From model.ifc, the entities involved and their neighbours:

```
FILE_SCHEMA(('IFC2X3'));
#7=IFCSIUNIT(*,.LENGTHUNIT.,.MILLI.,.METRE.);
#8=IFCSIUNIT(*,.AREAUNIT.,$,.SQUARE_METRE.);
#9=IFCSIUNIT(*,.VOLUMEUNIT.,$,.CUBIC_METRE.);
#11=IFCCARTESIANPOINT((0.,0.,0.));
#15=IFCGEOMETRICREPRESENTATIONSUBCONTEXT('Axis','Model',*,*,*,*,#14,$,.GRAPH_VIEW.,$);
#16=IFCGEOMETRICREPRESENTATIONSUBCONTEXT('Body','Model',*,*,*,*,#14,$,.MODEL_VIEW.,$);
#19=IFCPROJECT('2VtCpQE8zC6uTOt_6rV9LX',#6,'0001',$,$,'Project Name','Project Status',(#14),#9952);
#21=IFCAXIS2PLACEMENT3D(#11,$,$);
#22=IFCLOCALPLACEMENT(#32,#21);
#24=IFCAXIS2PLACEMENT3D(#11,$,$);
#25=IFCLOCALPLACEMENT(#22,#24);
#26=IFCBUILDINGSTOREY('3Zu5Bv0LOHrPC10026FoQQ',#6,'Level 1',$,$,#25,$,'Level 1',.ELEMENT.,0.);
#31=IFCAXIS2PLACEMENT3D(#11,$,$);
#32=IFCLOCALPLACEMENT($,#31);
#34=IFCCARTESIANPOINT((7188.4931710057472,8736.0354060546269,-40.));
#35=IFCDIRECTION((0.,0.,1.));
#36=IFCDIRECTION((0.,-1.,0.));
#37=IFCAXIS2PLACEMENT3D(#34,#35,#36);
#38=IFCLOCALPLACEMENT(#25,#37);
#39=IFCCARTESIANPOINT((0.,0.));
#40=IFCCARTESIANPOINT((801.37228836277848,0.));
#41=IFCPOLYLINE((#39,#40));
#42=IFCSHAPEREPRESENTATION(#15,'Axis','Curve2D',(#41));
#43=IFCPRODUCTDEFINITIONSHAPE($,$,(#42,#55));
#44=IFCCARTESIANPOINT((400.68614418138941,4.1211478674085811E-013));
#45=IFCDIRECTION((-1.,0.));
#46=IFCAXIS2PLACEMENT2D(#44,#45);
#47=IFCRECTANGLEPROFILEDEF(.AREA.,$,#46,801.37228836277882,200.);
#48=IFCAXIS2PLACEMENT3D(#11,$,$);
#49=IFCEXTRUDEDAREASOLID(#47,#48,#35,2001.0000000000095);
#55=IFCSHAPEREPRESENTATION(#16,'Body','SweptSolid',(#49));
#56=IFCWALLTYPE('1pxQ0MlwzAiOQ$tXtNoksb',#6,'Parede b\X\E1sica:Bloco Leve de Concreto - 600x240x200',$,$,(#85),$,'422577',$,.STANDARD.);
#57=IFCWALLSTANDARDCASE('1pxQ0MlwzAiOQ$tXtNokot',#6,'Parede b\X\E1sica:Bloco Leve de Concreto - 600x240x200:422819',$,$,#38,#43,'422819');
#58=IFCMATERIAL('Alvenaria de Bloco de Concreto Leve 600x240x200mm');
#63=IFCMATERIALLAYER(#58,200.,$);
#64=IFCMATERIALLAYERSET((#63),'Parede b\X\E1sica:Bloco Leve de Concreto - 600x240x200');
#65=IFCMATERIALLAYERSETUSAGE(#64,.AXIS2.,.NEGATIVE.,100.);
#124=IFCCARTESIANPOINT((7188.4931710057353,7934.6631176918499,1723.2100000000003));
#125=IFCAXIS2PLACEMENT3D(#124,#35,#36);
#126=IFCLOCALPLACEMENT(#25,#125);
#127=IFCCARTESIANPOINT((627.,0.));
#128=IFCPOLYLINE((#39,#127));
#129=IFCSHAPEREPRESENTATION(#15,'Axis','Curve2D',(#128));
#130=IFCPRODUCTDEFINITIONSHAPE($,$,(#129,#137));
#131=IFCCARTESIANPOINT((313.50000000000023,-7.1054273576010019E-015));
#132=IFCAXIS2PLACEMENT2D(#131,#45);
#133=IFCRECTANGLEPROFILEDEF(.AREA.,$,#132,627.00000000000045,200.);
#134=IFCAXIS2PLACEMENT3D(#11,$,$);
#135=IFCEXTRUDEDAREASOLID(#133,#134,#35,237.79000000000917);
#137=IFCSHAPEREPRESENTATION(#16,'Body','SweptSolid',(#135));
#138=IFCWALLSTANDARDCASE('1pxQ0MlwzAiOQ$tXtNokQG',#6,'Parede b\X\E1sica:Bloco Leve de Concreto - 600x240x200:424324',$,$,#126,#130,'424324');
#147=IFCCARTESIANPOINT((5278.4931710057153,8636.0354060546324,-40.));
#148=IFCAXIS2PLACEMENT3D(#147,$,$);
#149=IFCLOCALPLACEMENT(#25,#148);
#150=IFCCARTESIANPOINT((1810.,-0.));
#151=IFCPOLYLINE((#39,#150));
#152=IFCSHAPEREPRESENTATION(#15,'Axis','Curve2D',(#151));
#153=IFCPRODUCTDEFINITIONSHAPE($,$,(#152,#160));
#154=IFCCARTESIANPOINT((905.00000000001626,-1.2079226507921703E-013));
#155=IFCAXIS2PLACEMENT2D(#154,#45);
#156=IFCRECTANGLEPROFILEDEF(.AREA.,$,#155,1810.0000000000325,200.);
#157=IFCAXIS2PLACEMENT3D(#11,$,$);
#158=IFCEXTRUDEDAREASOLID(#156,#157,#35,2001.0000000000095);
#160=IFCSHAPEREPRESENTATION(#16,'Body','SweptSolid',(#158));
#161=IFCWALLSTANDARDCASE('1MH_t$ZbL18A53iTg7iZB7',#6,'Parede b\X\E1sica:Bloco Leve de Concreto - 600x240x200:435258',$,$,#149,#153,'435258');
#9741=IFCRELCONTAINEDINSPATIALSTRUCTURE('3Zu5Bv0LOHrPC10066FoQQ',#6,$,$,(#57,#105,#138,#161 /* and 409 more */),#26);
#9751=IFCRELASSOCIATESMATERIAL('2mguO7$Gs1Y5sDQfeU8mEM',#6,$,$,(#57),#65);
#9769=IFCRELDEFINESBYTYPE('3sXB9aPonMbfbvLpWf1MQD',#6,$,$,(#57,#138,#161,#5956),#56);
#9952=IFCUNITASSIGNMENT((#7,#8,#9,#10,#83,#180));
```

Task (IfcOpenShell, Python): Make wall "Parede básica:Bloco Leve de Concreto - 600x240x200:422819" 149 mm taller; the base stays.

```python
import ifcopenshell
import ifcopenshell.geom
import ifcopenshell.util.representation
import ifcopenshell.util.shape
import ifcopenshell.util.unit

model = ifcopenshell.open("model.ifc")
unit_scale = ifcopenshell.util.unit.calculate_unit_scale(model)
settings = ifcopenshell.geom.settings()


def volume(element):
    """Net volume in cubic metres, openings subtracted."""
    shape = ifcopenshell.geom.create_shape(settings, element)
    return ifcopenshell.util.shape.get_volume(shape.geometry)


wall = model.by_id(57)
before = volume(wall)

body = ifcopenshell.util.representation.get_representation(wall, "Model", "Body")
solid = body.Items[0]
old_height = solid.Depth
solid.Depth += 0.149 / unit_scale
after = volume(wall)

print(f"height {old_height:g} -> {solid.Depth:g}, volume {before:.3f} -> {after:.3f} m3")

model.write("model_v2.ifc")
```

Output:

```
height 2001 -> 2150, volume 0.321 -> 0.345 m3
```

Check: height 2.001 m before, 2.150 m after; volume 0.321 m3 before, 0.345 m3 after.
